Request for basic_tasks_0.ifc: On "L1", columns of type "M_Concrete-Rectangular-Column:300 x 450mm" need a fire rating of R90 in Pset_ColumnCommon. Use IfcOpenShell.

First a look at what the model holds.

```python
import ifcopenshell
import ifcopenshell.util.element

model = ifcopenshell.open("basic_tasks_0.ifc")
print(model.schema)
storey = next(s for s in model.by_type("IfcBuildingStorey") if s.Name == "L1")
columns = [e for e in ifcopenshell.util.element.get_decomposition(storey) if e.is_a("IfcColumn")]
seen = {}
for e in columns:
    element_type = ifcopenshell.util.element.get_type(e)
    key = (element_type.Name if element_type != e and element_type else None, ifcopenshell.util.element.get_pset(e, "Pset_ColumnCommon", "FireRating"))
    seen[key] = seen.get(key, 0) + 1
for (name, value), count in sorted(seen.items(), key=str):
    print(count, "x", name, "|", value)
```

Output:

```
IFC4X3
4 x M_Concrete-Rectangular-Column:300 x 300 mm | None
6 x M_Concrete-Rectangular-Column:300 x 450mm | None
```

```python
import ifcopenshell
import ifcopenshell.api.pset
import ifcopenshell.util.element

model = ifcopenshell.open("basic_tasks_0.ifc")

storey = next(s for s in model.by_type("IfcBuildingStorey") if s.Name == "L1")
columns = [e for e in ifcopenshell.util.element.get_decomposition(storey) if e.is_a("IfcColumn")]

count = 0
for e in columns:
    element_type = ifcopenshell.util.element.get_type(e)
    if element_type in (None, e) or element_type.Name != "M_Concrete-Rectangular-Column:300 x 450mm":
        continue
    # add_pset returns the element's existing set when there is one.
    pset = ifcopenshell.api.pset.add_pset(model, product=e, name="Pset_ColumnCommon")
    ifcopenshell.api.pset.edit_pset(model, pset=pset, properties={"FireRating": "R90"})
    count += 1

print(count, "columns updated")

model.write("basic_tasks_0_updated.ifc")
```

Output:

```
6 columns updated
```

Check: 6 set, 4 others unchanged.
